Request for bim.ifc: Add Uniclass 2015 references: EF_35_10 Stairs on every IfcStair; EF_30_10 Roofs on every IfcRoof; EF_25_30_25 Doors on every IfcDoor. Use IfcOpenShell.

First a look at what the model holds.

```python
import ifcopenshell

model = ifcopenshell.open("bim.ifc")
print(model.schema)
print("classifications:", [c.Name for c in model.by_type("IfcClassification")])
for ifc_class in ("IfcDoor", "IfcRoof", "IfcStair", "IfcWall", "IfcWindow"):
    print(ifc_class, len(model.by_type(ifc_class)))
```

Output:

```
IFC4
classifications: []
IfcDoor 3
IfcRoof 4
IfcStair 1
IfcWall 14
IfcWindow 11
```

```python
import ifcopenshell
import ifcopenshell.api.classification

model = ifcopenshell.open("bim.ifc")

system = ifcopenshell.api.classification.add_classification(model, classification="Uniclass 2015")

codes = {
    "IfcStair": ("EF_35_10", "Stairs"),
    "IfcRoof": ("EF_30_10", "Roofs"),
    "IfcDoor": ("EF_25_30_25", "Doors"),
}
for ifc_class, (code, name) in codes.items():
    products = model.by_type(ifc_class)
    ifcopenshell.api.classification.add_reference(
        model, products=products, classification=system, identification=code, name=name
    )
    print(code, len(products))

model.write("bim_v2.ifc")
```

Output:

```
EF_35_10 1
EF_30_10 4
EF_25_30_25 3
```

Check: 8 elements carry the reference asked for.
